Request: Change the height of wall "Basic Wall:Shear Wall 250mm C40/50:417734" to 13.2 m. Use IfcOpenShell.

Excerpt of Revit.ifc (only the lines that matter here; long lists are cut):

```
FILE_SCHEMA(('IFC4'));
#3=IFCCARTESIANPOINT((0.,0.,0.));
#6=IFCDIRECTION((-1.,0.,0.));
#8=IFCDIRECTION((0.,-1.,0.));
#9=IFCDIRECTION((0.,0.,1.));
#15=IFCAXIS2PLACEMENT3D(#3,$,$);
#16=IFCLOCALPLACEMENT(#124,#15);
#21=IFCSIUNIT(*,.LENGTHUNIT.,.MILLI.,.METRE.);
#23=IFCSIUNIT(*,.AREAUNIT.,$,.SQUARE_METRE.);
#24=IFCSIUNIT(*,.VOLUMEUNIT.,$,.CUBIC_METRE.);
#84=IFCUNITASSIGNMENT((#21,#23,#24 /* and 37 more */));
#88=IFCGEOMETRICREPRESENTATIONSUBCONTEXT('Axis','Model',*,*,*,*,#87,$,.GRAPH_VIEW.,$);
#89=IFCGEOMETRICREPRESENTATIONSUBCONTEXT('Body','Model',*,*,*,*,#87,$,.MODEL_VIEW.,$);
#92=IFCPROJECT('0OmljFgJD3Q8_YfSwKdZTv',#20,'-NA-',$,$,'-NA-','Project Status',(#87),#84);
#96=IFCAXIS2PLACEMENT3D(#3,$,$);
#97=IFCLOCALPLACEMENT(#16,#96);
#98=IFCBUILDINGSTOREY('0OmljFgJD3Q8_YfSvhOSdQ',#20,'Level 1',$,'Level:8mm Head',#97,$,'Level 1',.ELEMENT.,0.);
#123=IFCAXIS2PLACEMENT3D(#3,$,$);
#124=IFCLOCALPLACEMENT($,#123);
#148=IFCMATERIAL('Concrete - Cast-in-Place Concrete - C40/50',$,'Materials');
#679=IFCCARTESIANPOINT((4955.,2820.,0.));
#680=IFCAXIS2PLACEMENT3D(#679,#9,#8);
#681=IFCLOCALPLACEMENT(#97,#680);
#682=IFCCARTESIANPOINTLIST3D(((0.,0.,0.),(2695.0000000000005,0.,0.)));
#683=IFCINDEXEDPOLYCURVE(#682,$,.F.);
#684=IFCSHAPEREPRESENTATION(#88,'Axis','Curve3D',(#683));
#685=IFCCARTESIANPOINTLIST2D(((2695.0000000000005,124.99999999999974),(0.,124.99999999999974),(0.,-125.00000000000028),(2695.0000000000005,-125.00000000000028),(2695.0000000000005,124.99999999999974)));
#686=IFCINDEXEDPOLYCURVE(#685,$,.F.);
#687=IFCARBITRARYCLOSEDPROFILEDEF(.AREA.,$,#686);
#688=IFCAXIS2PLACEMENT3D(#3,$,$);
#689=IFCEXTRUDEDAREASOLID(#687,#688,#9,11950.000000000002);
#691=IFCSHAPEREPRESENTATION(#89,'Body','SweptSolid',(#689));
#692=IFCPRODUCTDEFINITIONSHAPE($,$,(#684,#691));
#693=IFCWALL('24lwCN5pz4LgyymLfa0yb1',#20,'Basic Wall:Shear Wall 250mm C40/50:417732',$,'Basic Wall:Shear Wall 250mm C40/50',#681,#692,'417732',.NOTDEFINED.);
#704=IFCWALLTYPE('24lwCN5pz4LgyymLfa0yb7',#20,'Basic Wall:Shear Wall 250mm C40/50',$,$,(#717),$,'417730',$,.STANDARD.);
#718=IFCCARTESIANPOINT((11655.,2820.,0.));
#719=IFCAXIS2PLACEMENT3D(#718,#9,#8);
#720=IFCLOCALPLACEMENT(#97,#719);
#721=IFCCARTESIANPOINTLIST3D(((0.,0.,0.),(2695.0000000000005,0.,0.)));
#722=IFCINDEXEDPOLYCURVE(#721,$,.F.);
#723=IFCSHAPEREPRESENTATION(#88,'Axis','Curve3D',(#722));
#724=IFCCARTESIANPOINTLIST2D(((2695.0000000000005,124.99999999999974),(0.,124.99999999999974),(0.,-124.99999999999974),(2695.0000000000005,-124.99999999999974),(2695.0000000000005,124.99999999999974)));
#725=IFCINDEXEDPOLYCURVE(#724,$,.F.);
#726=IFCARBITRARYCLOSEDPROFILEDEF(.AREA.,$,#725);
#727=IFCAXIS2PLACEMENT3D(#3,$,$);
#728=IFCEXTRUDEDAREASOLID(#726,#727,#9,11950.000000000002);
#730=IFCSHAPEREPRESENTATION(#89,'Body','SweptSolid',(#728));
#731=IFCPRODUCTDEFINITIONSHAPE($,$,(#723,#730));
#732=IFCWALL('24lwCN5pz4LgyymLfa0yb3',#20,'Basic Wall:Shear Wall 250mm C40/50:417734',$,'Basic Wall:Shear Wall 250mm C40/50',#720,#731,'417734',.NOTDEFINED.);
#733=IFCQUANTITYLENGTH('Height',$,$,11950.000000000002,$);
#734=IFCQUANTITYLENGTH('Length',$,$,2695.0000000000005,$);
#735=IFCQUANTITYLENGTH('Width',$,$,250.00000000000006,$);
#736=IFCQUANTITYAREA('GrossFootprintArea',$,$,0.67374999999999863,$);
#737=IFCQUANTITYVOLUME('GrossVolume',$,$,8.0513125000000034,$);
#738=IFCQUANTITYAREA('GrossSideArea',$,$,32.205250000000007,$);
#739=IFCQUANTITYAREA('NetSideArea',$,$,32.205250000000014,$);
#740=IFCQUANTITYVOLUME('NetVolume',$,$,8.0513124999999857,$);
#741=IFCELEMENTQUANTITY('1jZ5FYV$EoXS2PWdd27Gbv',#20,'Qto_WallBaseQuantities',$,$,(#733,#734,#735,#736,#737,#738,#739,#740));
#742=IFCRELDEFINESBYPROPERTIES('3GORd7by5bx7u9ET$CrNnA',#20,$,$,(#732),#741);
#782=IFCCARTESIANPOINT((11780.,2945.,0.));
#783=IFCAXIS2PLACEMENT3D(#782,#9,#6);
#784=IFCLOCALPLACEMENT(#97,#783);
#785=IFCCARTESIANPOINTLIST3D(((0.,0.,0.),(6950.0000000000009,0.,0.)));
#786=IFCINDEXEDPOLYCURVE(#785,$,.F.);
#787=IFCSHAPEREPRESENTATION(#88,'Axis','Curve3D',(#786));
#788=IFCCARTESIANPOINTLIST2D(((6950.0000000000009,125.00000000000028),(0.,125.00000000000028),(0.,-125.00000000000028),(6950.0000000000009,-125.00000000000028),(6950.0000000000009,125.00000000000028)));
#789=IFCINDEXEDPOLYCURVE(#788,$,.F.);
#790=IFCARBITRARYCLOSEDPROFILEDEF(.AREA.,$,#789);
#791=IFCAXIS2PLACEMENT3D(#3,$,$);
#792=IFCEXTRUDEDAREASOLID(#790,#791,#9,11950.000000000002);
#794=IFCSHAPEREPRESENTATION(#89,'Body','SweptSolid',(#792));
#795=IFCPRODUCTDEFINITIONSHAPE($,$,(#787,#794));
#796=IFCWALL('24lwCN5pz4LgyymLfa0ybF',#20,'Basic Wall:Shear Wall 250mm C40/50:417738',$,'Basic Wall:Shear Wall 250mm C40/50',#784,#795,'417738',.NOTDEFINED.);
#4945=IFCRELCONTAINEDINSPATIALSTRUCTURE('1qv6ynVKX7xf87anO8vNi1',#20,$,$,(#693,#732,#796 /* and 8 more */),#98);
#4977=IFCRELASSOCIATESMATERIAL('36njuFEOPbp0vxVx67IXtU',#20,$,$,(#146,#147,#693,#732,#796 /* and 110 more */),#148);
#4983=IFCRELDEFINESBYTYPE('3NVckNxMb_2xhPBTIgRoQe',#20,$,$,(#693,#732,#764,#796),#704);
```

```python
import ifcopenshell
import ifcopenshell.api.pset
import ifcopenshell.geom
import ifcopenshell.util.element
import ifcopenshell.util.representation
import ifcopenshell.util.shape
import ifcopenshell.util.unit

model = ifcopenshell.open("Revit.ifc")
unit_scale = ifcopenshell.util.unit.calculate_unit_scale(model)
area_scale = ifcopenshell.util.unit.calculate_unit_scale(model, "AREAUNIT")
volume_scale = ifcopenshell.util.unit.calculate_unit_scale(model, "VOLUMEUNIT")
settings = ifcopenshell.geom.settings()


def volume(element):
    """Net volume in cubic metres, openings subtracted."""
    shape = ifcopenshell.geom.create_shape(settings, element)
    return ifcopenshell.util.shape.get_volume(shape.geometry)


wall = model.by_guid("24lwCN5pz4LgyymLfa0yb3")
before = volume(wall)

body = ifcopenshell.util.representation.get_representation(wall, "Model", "Body")
solid = body.Items[0]
old_height = solid.Depth
solid.Depth = 13.2 / unit_scale
after = volume(wall)
thickness = 0.25  # wall thickness in metres

# Update the stored height, areas and volumes.
qto = model.by_id(ifcopenshell.util.element.get_pset(wall, "Qto_WallBaseQuantities", should_inherit=False)["id"])
ifcopenshell.api.pset.edit_qto(model, qto=qto, properties={
    "Height": solid.Depth,
    "GrossVolume": ifcopenshell.util.element.get_pset(wall, "Qto_WallBaseQuantities", "GrossVolume") * solid.Depth / old_height,
    "GrossSideArea": ifcopenshell.util.element.get_pset(wall, "Qto_WallBaseQuantities", "GrossSideArea") * solid.Depth / old_height,
    "NetSideArea": after / thickness / area_scale,
    "NetVolume": after / volume_scale,
})

print(f"height {old_height:g} -> {solid.Depth:g}, volume {before:.3f} -> {after:.3f} m3")

model.write("Revit_v2.ifc")
```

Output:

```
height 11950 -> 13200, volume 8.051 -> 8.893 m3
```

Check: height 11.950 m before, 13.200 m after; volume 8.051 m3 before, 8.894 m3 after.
